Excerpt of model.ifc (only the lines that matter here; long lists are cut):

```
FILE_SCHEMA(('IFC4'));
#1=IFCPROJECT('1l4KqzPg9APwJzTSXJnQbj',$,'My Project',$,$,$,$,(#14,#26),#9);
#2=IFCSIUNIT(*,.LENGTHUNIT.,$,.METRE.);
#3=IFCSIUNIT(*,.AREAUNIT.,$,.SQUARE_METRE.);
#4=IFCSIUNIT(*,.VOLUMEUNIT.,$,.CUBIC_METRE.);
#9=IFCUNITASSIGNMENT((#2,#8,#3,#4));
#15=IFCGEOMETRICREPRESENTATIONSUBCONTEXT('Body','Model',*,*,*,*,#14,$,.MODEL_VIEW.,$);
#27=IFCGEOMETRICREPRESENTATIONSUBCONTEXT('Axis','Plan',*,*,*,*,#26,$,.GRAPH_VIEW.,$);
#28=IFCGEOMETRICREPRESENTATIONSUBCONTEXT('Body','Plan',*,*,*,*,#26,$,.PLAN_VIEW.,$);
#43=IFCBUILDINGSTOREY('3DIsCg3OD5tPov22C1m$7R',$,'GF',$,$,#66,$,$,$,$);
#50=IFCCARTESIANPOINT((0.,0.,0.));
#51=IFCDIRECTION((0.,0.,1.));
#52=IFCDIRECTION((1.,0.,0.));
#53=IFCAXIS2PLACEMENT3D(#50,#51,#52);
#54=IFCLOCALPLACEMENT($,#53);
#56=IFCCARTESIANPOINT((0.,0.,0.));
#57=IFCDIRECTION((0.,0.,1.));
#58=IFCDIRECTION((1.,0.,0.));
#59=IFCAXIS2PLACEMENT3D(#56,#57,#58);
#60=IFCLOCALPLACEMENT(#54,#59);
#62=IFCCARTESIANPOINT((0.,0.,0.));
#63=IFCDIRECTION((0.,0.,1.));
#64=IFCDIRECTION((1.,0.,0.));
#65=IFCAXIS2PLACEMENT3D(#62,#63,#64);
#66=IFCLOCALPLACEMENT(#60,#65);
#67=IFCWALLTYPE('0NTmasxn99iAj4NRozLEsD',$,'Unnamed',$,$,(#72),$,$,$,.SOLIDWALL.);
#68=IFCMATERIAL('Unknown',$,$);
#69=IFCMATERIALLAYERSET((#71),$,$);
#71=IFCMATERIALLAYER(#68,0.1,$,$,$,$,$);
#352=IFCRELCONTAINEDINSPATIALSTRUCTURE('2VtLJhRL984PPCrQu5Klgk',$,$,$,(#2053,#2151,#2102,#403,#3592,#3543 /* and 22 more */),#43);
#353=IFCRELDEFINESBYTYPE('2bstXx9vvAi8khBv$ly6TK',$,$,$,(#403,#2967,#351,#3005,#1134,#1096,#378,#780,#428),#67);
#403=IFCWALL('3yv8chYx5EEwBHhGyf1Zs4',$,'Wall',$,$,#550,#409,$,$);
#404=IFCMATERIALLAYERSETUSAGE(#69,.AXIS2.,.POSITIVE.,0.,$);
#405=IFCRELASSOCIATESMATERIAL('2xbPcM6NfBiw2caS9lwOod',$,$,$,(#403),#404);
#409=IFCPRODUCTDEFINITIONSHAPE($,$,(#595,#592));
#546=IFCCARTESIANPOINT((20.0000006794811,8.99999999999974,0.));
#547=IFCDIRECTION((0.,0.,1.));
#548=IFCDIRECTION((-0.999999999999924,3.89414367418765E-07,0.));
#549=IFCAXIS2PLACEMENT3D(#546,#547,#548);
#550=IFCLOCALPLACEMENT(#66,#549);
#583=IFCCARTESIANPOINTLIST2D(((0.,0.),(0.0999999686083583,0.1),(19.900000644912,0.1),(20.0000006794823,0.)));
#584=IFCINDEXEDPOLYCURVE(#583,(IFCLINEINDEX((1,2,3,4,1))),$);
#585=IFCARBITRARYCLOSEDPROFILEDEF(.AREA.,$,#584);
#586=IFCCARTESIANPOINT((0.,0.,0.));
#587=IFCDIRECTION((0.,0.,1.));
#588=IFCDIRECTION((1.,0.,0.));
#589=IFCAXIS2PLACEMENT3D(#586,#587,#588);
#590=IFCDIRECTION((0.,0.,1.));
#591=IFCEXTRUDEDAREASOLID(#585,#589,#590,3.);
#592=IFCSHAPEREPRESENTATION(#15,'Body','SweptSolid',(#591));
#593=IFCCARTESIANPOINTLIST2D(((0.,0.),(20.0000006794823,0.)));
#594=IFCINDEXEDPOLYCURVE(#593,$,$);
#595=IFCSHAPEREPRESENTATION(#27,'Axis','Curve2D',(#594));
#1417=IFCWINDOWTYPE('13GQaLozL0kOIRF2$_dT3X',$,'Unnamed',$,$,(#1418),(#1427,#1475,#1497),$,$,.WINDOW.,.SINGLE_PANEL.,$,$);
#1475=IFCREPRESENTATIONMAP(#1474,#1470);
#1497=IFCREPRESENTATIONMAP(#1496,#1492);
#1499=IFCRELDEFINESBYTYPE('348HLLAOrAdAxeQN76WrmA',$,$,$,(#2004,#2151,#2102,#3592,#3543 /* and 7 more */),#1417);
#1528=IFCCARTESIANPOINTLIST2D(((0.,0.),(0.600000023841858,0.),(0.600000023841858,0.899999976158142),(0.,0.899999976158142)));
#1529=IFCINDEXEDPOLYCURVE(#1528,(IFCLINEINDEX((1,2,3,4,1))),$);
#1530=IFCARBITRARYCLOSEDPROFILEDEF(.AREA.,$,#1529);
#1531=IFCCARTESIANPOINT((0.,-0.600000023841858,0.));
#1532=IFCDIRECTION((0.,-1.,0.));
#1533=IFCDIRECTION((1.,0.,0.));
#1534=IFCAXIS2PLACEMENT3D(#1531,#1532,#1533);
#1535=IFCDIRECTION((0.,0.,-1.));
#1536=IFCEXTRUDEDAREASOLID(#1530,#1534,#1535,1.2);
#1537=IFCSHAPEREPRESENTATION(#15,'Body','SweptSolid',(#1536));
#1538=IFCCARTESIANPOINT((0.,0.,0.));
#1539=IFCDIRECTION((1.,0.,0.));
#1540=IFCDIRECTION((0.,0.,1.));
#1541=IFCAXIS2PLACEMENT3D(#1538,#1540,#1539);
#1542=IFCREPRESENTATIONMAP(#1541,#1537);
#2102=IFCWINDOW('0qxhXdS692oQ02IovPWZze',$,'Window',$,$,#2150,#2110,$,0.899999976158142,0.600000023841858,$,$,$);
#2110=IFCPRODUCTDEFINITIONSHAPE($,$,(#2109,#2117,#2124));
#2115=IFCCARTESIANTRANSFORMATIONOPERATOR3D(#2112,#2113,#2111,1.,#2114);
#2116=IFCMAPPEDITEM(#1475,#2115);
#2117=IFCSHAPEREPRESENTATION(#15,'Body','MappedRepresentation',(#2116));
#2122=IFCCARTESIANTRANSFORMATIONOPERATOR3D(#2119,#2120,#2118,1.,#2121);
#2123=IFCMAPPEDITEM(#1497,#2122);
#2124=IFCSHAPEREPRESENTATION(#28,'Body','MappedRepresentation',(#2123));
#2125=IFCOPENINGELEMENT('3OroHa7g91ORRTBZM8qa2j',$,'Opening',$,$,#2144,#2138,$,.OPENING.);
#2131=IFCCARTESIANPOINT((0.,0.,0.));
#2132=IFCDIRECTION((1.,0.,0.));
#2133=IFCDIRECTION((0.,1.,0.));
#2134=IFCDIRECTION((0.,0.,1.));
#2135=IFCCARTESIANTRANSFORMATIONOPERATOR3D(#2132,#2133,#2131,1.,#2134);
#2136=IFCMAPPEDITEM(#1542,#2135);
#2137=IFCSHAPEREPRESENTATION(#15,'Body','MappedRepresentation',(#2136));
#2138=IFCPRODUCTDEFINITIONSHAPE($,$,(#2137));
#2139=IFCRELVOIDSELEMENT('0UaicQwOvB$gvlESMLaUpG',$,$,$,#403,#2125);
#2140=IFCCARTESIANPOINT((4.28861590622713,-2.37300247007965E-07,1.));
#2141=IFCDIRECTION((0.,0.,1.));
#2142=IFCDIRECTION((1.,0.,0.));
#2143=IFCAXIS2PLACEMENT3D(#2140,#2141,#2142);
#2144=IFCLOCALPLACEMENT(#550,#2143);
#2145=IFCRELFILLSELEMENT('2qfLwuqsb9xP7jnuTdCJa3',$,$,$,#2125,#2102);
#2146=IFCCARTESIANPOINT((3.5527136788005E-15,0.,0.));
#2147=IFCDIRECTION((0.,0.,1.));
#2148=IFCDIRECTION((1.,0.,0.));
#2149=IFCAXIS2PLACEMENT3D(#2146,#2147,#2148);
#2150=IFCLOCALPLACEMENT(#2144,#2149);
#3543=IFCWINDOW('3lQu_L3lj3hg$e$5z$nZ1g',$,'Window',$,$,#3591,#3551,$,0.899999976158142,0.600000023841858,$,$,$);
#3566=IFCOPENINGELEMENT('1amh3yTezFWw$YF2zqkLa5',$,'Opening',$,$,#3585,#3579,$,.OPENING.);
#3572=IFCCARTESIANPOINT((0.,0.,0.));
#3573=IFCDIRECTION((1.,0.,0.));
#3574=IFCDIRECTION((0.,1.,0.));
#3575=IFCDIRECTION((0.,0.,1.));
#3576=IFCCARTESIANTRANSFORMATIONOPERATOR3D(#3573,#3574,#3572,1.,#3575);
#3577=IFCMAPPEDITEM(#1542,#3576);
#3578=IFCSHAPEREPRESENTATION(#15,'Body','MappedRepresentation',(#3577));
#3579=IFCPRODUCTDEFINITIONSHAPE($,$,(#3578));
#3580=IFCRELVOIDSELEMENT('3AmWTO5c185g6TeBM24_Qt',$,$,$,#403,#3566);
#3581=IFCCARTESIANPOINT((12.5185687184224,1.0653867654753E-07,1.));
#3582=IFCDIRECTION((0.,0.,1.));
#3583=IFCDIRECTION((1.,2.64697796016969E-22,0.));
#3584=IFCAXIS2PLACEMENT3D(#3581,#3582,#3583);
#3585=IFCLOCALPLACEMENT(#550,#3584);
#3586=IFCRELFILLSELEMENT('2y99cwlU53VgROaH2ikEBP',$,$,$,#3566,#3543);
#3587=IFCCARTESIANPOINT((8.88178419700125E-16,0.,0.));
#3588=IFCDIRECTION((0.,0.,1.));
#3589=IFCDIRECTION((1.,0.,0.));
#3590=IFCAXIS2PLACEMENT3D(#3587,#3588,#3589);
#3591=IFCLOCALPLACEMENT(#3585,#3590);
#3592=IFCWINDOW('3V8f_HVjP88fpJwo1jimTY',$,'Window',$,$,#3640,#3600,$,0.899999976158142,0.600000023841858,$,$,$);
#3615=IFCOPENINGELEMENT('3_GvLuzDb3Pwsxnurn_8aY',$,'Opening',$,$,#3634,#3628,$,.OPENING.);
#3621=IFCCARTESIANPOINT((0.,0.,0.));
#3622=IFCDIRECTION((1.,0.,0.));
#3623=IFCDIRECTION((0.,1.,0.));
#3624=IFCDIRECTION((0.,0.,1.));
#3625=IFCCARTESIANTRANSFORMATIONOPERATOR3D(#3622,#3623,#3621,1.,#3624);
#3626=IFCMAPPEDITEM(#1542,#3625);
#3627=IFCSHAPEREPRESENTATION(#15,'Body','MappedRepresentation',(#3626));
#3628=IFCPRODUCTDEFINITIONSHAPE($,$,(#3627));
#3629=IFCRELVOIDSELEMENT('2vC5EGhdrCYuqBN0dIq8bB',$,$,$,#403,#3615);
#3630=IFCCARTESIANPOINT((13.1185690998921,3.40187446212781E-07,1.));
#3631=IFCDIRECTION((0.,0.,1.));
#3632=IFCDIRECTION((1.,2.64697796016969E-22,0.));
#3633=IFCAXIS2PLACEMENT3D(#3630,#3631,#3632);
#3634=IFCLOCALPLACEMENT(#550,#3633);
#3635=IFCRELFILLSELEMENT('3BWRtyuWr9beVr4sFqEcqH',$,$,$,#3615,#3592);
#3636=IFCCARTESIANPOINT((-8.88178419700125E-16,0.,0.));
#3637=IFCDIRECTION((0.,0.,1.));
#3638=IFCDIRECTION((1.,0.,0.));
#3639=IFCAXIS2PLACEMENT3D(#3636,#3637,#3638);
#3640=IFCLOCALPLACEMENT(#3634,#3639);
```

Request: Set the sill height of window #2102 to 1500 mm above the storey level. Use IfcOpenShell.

```python
import numpy as np
import ifcopenshell
import ifcopenshell.api.geometry
import ifcopenshell.geom
import ifcopenshell.util.element
import ifcopenshell.util.placement
import ifcopenshell.util.shape
import ifcopenshell.util.unit

model = ifcopenshell.open("model.ifc")
unit_scale = ifcopenshell.util.unit.calculate_unit_scale(model)

window = model.by_guid("0qxhXdS692oQ02IovPWZze")
opening = window.FillsVoids[0].RelatingOpeningElement
storey = ifcopenshell.util.element.get_container(window, ifc_class="IfcBuildingStorey")
level = ifcopenshell.util.placement.get_local_placement(storey.ObjectPlacement)[2, 3]

# The opening's origin need not be at the sill, so measure its lowest point.
shape = ifcopenshell.geom.create_shape(ifcopenshell.geom.settings(), opening)
bottom = ifcopenshell.util.shape.get_shape_bottom_elevation(shape, shape.geometry) / unit_scale
dz = level + 1.5 / unit_scale - bottom

shift = np.array([0.0, 0.0, dz])
# The window is placed relative to its opening, so it follows when the opening moves.
matrix = ifcopenshell.util.placement.get_local_placement(opening.ObjectPlacement)
matrix[:3, 3] += shift
ifcopenshell.api.geometry.edit_object_placement(
    model, product=opening, matrix=matrix, is_si=False, should_transform_children=True
)

print(f"moved by {dz * unit_scale:+.3f} m")

model.write("model_edited.ifc")
```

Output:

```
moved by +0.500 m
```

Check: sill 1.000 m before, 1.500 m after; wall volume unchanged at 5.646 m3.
